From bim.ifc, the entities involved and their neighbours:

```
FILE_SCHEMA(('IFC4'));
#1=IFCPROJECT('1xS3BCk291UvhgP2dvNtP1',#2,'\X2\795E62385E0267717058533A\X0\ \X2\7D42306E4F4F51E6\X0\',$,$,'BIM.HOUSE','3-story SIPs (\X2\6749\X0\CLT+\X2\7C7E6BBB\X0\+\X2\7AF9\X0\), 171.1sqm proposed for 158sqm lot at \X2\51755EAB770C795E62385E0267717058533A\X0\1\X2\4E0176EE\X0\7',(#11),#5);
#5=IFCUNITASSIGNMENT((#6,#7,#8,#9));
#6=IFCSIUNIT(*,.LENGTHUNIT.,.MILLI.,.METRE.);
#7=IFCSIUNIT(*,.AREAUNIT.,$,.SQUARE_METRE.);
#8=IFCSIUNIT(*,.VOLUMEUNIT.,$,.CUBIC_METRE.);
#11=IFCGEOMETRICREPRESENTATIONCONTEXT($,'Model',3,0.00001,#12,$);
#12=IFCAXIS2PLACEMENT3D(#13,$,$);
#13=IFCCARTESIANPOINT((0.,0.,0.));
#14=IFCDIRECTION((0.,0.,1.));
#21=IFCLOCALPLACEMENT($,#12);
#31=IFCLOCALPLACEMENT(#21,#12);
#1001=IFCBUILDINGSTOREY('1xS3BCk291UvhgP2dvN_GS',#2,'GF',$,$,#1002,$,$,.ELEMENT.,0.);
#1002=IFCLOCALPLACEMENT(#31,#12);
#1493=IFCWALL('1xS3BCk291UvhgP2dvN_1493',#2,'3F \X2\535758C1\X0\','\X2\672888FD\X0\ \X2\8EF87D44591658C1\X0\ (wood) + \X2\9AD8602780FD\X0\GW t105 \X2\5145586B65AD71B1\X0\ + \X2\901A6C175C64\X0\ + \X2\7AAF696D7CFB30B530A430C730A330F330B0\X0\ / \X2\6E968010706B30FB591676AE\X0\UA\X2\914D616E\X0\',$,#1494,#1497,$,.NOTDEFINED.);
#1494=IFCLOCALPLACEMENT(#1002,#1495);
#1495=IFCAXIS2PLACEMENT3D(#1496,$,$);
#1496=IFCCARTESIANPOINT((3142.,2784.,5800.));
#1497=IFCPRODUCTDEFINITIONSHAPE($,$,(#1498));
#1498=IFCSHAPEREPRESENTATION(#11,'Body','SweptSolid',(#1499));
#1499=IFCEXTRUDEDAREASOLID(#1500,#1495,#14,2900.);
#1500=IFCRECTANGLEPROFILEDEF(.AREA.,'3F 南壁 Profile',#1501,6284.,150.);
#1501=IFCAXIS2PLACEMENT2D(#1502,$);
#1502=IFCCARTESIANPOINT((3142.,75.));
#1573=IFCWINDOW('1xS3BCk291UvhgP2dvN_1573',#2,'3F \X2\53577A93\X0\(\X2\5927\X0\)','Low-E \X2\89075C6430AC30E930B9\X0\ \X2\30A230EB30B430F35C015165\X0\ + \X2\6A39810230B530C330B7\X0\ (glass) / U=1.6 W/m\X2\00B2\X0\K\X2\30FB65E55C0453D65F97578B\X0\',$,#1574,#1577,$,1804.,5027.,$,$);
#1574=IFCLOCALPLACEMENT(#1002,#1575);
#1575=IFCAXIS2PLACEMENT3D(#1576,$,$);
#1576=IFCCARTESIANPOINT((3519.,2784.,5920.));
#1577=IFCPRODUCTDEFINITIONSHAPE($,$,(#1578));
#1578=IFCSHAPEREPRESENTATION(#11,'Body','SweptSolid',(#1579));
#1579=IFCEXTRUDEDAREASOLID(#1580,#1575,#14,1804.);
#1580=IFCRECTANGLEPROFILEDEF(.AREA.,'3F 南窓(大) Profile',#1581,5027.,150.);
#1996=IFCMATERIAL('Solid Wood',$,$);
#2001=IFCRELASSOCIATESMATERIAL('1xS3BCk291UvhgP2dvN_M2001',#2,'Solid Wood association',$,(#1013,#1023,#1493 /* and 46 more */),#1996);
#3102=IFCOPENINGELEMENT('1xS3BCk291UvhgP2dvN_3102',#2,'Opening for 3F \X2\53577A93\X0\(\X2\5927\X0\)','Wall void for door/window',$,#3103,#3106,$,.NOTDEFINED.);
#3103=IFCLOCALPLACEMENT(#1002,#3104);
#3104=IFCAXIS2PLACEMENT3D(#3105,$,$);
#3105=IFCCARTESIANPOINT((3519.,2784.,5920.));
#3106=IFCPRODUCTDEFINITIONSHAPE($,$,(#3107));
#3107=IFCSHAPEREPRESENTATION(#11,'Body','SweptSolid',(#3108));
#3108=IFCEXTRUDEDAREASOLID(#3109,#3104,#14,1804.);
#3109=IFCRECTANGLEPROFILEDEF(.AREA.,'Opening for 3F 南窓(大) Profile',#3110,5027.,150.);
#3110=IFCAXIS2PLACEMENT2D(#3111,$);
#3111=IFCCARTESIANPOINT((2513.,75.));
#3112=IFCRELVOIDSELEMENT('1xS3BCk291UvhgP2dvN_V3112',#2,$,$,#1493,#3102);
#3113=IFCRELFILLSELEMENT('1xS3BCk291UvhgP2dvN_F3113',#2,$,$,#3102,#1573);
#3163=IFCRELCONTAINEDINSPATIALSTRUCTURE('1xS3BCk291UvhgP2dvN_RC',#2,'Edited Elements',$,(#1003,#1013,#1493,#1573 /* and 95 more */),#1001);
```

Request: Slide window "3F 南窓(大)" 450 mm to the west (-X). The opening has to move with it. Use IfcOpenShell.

```python
import ifcopenshell
import ifcopenshell.api.geometry
import ifcopenshell.util.placement
import ifcopenshell.util.unit

model = ifcopenshell.open("bim.ifc")
unit_scale = ifcopenshell.util.unit.calculate_unit_scale(model)

window = model.by_id(1573)
opening = window.FillsVoids[0].RelatingOpeningElement
wall = opening.VoidsElements[0].RelatingBuildingElement

wall_matrix = ifcopenshell.util.placement.get_local_placement(wall.ObjectPlacement)
shift = wall_matrix[:3, 0] * -0.45 / unit_scale
before = ifcopenshell.util.placement.get_local_placement(window.ObjectPlacement)[:3, 3].copy()

# The window is not placed relative to its opening, so move both.
for product in (opening, window):
    matrix = ifcopenshell.util.placement.get_local_placement(product.ObjectPlacement)
    matrix[:3, 3] += shift
    ifcopenshell.api.geometry.edit_object_placement(model, product=product, matrix=matrix, is_si=False)

after = ifcopenshell.util.placement.get_local_placement(window.ObjectPlacement)[:3, 3]
print("window moved by", (after - before).round(3) + 0.0)

model.write("bim-out.ifc")
```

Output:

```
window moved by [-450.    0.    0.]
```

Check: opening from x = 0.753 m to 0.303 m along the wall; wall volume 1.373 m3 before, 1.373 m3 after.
